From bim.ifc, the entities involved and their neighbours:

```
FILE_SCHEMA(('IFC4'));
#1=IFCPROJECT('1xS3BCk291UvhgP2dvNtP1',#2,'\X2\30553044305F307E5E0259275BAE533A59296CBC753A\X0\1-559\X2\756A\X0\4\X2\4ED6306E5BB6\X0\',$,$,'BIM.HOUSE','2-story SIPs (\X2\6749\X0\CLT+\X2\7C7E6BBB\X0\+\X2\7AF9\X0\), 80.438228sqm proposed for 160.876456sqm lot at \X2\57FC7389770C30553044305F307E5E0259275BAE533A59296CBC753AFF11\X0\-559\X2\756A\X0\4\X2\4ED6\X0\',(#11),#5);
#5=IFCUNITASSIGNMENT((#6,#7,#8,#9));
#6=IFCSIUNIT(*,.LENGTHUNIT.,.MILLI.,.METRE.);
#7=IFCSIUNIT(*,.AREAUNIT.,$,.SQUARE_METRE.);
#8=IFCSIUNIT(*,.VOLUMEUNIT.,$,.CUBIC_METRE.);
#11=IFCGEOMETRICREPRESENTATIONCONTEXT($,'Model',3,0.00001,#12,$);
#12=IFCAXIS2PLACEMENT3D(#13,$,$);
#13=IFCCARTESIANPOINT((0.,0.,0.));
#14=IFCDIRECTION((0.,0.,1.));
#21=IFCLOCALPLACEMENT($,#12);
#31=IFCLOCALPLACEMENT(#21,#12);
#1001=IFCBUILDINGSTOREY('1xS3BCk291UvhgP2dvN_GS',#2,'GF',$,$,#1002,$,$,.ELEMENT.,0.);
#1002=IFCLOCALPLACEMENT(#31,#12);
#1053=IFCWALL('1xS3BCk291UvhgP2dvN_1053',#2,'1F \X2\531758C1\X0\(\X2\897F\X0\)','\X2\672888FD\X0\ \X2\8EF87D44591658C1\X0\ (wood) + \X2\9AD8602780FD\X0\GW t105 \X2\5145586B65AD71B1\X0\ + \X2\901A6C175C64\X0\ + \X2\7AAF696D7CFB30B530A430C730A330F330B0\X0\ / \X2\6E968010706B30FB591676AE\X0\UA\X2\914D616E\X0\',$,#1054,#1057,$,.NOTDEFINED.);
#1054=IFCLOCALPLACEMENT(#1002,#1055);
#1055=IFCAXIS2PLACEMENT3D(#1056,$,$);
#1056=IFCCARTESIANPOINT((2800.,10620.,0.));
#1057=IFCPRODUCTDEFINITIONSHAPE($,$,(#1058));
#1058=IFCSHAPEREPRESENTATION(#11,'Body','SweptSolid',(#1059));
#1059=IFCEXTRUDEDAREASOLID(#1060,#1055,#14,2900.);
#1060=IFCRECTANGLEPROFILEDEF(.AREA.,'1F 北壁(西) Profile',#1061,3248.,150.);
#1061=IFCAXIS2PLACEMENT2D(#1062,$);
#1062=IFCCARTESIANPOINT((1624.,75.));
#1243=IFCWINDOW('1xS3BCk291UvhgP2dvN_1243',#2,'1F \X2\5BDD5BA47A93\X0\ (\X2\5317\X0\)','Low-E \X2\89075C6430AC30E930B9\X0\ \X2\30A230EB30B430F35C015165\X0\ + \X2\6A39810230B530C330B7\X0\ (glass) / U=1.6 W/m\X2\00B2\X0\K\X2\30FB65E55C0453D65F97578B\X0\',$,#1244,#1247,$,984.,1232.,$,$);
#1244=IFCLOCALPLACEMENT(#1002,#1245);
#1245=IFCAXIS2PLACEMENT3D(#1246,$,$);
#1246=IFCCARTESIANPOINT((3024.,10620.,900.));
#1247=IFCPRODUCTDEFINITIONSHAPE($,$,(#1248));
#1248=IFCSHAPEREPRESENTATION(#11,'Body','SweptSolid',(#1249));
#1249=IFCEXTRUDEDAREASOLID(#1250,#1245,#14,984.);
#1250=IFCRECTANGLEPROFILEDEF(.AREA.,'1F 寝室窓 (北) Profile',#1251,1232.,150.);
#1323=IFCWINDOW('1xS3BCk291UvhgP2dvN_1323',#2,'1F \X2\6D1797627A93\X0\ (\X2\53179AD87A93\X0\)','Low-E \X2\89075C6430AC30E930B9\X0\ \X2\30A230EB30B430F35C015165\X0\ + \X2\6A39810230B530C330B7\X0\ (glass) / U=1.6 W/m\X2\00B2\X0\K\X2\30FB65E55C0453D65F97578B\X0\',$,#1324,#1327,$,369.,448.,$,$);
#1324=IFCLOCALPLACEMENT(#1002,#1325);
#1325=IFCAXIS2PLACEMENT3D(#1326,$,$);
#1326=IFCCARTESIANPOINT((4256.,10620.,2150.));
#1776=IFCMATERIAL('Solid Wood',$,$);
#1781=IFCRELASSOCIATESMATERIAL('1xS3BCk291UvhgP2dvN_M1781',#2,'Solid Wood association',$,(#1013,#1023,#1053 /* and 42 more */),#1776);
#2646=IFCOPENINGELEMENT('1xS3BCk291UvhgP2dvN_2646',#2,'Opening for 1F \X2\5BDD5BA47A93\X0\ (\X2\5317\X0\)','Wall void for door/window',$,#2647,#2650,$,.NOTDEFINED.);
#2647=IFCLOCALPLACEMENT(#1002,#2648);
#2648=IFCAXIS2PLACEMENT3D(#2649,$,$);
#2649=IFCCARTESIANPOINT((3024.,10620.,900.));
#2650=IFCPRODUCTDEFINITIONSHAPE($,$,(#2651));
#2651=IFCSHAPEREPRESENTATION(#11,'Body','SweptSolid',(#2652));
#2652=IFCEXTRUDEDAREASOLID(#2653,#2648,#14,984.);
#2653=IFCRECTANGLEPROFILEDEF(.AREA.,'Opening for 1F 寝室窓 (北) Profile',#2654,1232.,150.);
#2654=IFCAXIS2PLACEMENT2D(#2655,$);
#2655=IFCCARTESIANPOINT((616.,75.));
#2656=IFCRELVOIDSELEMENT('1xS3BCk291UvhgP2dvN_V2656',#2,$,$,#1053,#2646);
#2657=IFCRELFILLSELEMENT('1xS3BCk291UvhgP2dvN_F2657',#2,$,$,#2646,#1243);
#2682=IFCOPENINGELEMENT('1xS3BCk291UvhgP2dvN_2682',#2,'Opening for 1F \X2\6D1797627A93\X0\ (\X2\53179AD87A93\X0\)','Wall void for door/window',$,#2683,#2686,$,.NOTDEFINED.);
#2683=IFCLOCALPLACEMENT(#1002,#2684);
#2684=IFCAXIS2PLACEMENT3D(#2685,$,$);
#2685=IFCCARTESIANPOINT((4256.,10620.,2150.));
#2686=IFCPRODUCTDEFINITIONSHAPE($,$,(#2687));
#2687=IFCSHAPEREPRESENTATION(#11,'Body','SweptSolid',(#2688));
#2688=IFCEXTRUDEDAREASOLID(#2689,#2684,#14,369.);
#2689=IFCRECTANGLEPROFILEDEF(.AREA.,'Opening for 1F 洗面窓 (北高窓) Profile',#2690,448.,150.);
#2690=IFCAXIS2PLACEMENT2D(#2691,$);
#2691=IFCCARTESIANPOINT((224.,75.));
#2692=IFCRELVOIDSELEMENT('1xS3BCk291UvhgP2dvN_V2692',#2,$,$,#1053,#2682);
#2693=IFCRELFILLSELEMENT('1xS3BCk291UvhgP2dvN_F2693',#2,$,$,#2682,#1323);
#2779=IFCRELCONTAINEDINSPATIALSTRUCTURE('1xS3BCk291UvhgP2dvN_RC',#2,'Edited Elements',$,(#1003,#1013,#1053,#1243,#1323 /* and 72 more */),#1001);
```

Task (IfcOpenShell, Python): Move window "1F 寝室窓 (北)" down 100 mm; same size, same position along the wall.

```python
import numpy as np
import ifcopenshell
import ifcopenshell.api.geometry
import ifcopenshell.util.placement
import ifcopenshell.util.unit

model = ifcopenshell.open("bim.ifc")
unit_scale = ifcopenshell.util.unit.calculate_unit_scale(model)

window = model.by_id(1243)
opening = window.FillsVoids[0].RelatingOpeningElement
dz = -0.1 / unit_scale

shift = np.array([0.0, 0.0, dz])
# The window is not placed relative to its opening, so move both.
for product in (opening, window):
    matrix = ifcopenshell.util.placement.get_local_placement(product.ObjectPlacement)
    matrix[:3, 3] += shift
    ifcopenshell.api.geometry.edit_object_placement(model, product=product, matrix=matrix, is_si=False)

print(f"moved by {dz * unit_scale:+.3f} m")

model.write("bim_edited.ifc")
```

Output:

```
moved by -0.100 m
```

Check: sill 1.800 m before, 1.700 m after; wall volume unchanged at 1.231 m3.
